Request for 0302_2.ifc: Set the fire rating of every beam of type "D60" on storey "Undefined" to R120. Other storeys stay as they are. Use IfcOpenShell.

First a look at what the model holds.

```python
import ifcopenshell
import ifcopenshell.util.element

model = ifcopenshell.open("0302_2.ifc")
print(model.schema)
storey = next(s for s in model.by_type("IfcBuildingStorey") if s.Name == "Undefined")
beams = [e for e in ifcopenshell.util.element.get_decomposition(storey) if e.is_a("IfcBeam")]
seen = {}
for e in beams:
    element_type = ifcopenshell.util.element.get_type(e)
    key = (element_type.Name if element_type != e and element_type else None, ifcopenshell.util.element.get_pset(e, "Pset_BeamCommon", "FireRating"))
    seen[key] = seen.get(key, 0) + 1
for (name, value), count in sorted(seen.items(), key=str):
    print(count, "x", name, "|", value)
```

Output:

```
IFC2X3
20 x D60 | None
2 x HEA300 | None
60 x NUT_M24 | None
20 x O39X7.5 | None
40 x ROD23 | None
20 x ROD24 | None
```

```python
import ifcopenshell
import ifcopenshell.api.pset
import ifcopenshell.util.element

model = ifcopenshell.open("0302_2.ifc")

storey = next(s for s in model.by_type("IfcBuildingStorey") if s.Name == "Undefined")
beams = [e for e in ifcopenshell.util.element.get_decomposition(storey) if e.is_a("IfcBeam")]

count = 0
for e in beams:
    element_type = ifcopenshell.util.element.get_type(e)
    if element_type in (None, e) or element_type.Name != "D60":
        continue
    found = ifcopenshell.util.element.get_pset(e, "Pset_BeamCommon", should_inherit=False)
    if found:
        pset = model.by_id(found["id"])
        if len(ifcopenshell.util.element.get_elements_by_pset(pset)) > 1:
            pset = ifcopenshell.api.pset.unshare_pset(model, products=[e], pset=pset)[0]
    else:
        pset = ifcopenshell.api.pset.add_pset(model, product=e, name="Pset_BeamCommon")
    ifcopenshell.api.pset.edit_pset(model, pset=pset, properties={"FireRating": "R120"})
    count += 1

print(count, "beams updated")

model.write("0302_2_v2.ifc")
```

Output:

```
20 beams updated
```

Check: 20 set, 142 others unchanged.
